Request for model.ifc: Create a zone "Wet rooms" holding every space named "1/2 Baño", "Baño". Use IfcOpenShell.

First a look at what the model holds.

```python
import ifcopenshell

model = ifcopenshell.open("model.ifc")
print(model.schema)
seen = {}
for space in model.by_type("IfcSpace"):
    seen[space.LongName] = seen.get(space.LongName, 0) + 1
for name, count in sorted(seen.items(), key=str):
    print(count, "x", name)
print("zones:", [z.Name for z in model.by_type("IfcZone")][:20])
```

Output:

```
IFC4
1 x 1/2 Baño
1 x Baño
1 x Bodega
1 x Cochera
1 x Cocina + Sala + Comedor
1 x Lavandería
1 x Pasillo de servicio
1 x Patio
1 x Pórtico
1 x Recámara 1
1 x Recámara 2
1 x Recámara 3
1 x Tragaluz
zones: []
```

```python
import ifcopenshell
import ifcopenshell.api.group
import ifcopenshell.api.root

model = ifcopenshell.open("model.ifc")

names = {"1/2 Baño", "Baño"}
spaces = [s for s in model.by_type("IfcSpace") if s.LongName in names]

zone = ifcopenshell.api.root.create_entity(model, ifc_class="IfcZone", name="Wet rooms")
ifcopenshell.api.group.assign_group(model, products=spaces, group=zone)
print(len(spaces), "spaces in", zone.Name)

model.write("model_edited.ifc")
```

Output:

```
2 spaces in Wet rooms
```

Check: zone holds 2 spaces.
